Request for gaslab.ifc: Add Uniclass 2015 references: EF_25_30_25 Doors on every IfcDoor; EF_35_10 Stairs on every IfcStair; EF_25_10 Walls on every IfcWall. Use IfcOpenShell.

First a look at what the model holds.

```python
import ifcopenshell

model = ifcopenshell.open("gaslab.ifc")
print(model.schema)
print("classifications:", [c.Name for c in model.by_type("IfcClassification")])
for ifc_class in ("IfcDoor", "IfcRoof", "IfcStair", "IfcWall", "IfcWindow"):
    print(ifc_class, len(model.by_type(ifc_class)))
```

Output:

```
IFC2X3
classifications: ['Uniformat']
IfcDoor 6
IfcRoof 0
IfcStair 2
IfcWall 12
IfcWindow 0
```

```python
import ifcopenshell
import ifcopenshell.api.classification

model = ifcopenshell.open("gaslab.ifc")

# IFC2X3 requires Source and Edition and has no link from the project to the system.
system = model.create_entity("IfcClassification", Source="NBS", Edition="2015", Name="Uniclass 2015")

codes = {
    "IfcDoor": ("EF_25_30_25", "Doors"),
    "IfcStair": ("EF_35_10", "Stairs"),
    "IfcWall": ("EF_25_10", "Walls"),
}
for ifc_class, (code, name) in codes.items():
    products = model.by_type(ifc_class)
    ifcopenshell.api.classification.add_reference(
        model, products=products, classification=system, identification=code, name=name
    )
    print(code, len(products))

model.write("gaslab-out.ifc")
```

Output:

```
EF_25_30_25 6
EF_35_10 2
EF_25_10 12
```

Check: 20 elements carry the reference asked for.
